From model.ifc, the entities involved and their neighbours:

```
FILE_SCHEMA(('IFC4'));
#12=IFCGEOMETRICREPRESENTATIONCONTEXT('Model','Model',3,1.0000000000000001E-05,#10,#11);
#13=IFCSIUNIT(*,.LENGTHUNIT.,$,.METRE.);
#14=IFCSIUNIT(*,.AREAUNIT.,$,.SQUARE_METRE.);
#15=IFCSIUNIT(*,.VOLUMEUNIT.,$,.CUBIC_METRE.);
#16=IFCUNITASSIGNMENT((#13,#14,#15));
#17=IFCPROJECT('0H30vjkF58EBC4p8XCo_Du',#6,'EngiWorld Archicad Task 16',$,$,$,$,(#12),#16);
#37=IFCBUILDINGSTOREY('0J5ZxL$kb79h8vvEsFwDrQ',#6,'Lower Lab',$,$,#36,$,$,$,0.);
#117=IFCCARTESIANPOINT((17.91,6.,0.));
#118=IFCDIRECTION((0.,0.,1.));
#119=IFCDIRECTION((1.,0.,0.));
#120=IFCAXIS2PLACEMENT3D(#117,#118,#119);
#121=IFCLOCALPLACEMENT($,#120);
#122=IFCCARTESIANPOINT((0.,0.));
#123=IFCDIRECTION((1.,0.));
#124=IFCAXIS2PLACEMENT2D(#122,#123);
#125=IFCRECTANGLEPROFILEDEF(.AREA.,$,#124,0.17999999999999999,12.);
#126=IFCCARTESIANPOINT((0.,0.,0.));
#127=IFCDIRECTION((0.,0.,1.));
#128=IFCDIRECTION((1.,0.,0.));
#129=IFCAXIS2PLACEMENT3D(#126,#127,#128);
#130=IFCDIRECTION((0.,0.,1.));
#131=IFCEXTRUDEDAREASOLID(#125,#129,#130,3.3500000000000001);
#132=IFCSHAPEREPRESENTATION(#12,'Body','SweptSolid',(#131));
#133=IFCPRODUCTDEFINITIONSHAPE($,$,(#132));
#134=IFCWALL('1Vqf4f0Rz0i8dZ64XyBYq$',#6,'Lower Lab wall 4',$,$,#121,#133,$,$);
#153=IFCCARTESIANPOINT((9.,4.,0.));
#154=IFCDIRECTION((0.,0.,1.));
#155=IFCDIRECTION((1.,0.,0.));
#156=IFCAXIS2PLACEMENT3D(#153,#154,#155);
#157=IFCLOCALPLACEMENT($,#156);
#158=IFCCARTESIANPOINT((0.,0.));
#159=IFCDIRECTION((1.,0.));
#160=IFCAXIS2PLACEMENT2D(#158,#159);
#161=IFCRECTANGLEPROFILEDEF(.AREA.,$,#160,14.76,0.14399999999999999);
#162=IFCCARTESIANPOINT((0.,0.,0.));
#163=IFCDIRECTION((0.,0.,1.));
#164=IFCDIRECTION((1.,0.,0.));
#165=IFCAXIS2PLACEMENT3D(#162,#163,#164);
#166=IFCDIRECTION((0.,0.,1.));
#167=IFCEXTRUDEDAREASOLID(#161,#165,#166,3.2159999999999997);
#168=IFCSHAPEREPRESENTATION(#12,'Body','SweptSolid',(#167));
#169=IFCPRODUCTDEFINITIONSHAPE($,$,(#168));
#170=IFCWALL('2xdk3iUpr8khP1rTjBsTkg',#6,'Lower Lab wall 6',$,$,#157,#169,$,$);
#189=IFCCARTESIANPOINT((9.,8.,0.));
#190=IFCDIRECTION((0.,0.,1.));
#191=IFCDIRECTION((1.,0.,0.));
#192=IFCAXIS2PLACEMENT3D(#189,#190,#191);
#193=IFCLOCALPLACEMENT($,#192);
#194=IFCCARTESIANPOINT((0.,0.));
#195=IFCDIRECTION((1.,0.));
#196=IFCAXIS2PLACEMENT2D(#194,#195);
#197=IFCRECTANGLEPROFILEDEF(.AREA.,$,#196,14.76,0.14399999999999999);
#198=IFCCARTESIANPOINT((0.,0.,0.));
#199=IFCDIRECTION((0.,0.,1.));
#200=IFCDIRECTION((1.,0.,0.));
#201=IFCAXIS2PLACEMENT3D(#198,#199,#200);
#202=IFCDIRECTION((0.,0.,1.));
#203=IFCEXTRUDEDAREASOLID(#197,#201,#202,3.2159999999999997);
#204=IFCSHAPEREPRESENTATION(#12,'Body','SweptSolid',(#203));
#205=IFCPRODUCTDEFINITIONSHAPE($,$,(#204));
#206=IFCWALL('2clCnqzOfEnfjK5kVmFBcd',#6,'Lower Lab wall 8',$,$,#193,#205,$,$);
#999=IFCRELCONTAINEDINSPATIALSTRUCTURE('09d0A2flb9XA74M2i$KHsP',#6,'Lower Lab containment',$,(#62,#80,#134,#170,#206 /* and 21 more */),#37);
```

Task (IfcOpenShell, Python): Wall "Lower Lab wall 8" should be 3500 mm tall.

```python
import ifcopenshell
import ifcopenshell.geom
import ifcopenshell.util.shape
import ifcopenshell.util.unit

model = ifcopenshell.open("model.ifc")
unit_scale = ifcopenshell.util.unit.calculate_unit_scale(model)
settings = ifcopenshell.geom.settings()


def volume(element):
    """Net volume in cubic metres, openings subtracted."""
    shape = ifcopenshell.geom.create_shape(settings, element)
    return ifcopenshell.util.shape.get_volume(shape.geometry)


wall = model.by_guid("2clCnqzOfEnfjK5kVmFBcd")
before = volume(wall)

body = next(r for r in wall.Representation.Representations if r.RepresentationIdentifier == "Body")
solid = body.Items[0]
old_height = solid.Depth
solid.Depth = 3.5 / unit_scale
after = volume(wall)

print(f"height {old_height:g} -> {solid.Depth:g}, volume {before:.3f} -> {after:.3f} m3")

model.write("model_rev.ifc")
```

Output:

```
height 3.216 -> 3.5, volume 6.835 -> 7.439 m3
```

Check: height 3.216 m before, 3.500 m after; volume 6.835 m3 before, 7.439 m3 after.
